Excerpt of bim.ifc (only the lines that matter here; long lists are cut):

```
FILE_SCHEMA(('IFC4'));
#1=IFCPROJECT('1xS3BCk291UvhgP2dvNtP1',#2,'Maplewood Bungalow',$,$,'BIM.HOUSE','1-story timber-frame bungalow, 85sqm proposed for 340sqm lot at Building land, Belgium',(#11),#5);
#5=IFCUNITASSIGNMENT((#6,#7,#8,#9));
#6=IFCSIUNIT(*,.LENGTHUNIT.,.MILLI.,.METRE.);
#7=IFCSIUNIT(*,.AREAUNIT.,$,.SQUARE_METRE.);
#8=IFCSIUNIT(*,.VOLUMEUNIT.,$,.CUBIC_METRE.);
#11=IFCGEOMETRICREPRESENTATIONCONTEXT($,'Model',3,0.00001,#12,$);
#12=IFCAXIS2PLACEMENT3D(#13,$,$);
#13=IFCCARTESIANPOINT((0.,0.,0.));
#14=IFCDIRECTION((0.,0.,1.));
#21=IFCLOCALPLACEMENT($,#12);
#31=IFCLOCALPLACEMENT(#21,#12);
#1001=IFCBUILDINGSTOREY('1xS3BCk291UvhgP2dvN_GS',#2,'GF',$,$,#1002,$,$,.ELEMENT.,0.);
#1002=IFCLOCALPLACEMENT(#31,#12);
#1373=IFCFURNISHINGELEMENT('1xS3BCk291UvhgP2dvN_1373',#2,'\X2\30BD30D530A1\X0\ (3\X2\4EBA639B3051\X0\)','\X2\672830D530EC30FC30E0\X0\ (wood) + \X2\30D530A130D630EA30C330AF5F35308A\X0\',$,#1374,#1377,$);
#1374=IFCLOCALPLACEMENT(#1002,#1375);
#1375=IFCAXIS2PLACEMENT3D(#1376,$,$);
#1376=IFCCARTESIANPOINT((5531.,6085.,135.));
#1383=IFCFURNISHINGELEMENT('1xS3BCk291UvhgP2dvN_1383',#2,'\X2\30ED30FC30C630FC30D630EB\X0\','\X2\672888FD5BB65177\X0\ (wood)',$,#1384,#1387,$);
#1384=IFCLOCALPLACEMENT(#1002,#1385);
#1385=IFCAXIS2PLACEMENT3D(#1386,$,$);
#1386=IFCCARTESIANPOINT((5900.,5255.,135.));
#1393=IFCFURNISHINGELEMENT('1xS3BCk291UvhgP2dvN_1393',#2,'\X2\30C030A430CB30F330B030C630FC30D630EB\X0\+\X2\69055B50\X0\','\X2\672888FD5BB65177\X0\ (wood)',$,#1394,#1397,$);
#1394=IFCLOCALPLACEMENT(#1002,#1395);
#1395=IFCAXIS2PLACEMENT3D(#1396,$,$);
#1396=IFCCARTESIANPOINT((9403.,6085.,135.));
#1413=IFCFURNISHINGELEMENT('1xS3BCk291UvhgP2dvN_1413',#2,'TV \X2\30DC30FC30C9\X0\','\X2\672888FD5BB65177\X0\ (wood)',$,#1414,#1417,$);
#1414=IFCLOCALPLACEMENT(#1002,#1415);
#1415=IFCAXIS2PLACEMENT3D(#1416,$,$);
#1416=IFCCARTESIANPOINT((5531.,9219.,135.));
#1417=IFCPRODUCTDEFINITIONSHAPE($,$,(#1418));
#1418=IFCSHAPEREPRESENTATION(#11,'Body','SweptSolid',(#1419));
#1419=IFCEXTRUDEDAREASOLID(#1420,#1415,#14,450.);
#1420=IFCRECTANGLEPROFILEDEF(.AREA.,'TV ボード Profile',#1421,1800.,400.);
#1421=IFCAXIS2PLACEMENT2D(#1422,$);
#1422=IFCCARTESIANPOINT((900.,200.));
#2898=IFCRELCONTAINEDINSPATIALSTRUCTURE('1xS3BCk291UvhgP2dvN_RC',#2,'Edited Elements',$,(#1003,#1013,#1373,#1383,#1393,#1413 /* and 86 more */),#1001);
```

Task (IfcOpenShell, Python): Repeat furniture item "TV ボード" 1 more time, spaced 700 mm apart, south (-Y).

```python
import numpy as np
import ifcopenshell
import ifcopenshell.api.geometry
import ifcopenshell.api.root
import ifcopenshell.util.element
import ifcopenshell.util.placement
import ifcopenshell.util.unit

model = ifcopenshell.open("bim.ifc")
unit_scale = ifcopenshell.util.unit.calculate_unit_scale(model)


def reuse_history(source, copy):
    """copy_class also copies each property set's owner history, people and application; keep the originals."""
    for rel in copy.IsDefinedBy:
        if rel.is_a("IfcRelDefinesByProperties") and (history := rel.RelatingPropertyDefinition.OwnerHistory):
            rel.RelatingPropertyDefinition.OwnerHistory = source.OwnerHistory
            ifcopenshell.util.element.remove_deep2(model, history)


source = model.by_id(1413)
base = ifcopenshell.util.placement.get_local_placement(source.ObjectPlacement)
step = np.array([0.0, -1.0, 0.0]) * 0.7 / unit_scale

for i in range(1, 2):
    copy = ifcopenshell.api.root.copy_class(model, product=source)
    copy.Representation = ifcopenshell.util.element.copy_deep(
        model, source.Representation, exclude=["IfcGeometricRepresentationContext", "IfcRepresentationMap"]
    )
    reuse_history(source, copy)
    matrix = base.copy()
    matrix[:3, 3] += i * step
    print("added at", matrix[:3, 3].round(3) + 0.0)
    ifcopenshell.api.geometry.edit_object_placement(model, product=copy, matrix=matrix, is_si=False)

model.write("bim-out.ifc")
```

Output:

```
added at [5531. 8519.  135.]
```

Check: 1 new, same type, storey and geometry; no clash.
